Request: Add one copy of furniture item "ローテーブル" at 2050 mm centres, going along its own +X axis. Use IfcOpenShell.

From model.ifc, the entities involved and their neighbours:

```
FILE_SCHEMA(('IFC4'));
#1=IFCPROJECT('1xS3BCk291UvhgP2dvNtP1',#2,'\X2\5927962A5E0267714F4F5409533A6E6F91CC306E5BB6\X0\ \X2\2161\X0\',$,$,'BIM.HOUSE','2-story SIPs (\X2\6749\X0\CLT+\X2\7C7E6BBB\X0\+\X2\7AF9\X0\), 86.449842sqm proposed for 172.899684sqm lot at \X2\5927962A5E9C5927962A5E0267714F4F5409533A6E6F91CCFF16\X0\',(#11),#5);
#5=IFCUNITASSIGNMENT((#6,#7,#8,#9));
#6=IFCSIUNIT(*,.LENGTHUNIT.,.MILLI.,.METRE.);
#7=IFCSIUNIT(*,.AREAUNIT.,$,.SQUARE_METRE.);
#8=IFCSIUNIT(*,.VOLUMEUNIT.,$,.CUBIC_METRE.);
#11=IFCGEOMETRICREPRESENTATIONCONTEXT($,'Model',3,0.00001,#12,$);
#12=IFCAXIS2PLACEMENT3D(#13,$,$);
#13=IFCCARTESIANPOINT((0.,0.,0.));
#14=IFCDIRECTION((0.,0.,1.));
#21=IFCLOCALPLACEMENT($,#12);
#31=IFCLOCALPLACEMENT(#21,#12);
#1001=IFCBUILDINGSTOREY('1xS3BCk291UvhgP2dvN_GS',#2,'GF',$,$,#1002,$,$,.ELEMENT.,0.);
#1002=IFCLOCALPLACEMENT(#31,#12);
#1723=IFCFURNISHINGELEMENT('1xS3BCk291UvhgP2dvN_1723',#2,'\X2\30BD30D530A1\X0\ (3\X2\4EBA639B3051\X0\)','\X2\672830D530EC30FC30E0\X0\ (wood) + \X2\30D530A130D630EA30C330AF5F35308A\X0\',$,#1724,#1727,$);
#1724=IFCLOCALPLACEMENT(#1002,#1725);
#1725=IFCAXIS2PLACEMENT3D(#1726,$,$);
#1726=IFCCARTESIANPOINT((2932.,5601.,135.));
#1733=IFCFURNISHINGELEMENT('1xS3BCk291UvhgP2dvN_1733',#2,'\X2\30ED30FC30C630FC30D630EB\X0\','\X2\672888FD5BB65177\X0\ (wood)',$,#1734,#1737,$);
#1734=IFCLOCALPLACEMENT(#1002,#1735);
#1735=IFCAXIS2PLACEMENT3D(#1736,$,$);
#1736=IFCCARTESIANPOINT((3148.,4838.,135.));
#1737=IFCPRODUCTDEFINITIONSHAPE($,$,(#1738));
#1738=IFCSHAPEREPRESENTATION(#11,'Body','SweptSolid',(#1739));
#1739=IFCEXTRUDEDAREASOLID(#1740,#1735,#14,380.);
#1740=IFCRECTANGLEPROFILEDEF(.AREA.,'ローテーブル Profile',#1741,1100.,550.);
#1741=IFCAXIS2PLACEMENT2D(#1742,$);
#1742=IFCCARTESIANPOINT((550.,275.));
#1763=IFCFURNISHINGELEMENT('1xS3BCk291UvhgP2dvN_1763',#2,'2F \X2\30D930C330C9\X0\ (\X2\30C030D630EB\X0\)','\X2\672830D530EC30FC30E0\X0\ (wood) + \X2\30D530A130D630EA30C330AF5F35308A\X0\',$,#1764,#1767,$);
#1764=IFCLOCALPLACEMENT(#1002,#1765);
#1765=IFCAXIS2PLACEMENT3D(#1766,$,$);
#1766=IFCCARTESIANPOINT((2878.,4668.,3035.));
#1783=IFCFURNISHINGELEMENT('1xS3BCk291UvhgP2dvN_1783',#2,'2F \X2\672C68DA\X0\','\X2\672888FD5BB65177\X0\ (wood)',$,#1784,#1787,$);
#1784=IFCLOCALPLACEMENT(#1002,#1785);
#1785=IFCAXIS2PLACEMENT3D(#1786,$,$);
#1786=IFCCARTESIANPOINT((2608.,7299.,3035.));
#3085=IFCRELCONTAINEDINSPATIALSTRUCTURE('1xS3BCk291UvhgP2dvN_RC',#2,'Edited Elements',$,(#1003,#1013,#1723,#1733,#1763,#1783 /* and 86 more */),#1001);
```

```python
import ifcopenshell
import ifcopenshell.api.geometry
import ifcopenshell.api.root
import ifcopenshell.util.element
import ifcopenshell.util.placement

model = ifcopenshell.open("model.ifc")


def reuse_history(source, copy):
    """copy_class also copies each property set's owner history, people and application; keep the originals."""
    for rel in copy.IsDefinedBy:
        if rel.is_a("IfcRelDefinesByProperties") and (history := rel.RelatingPropertyDefinition.OwnerHistory):
            rel.RelatingPropertyDefinition.OwnerHistory = source.OwnerHistory
            ifcopenshell.util.element.remove_deep2(model, history)


source = model.by_id(1733)
base = ifcopenshell.util.placement.get_local_placement(source.ObjectPlacement)
step = base[:3, 0] * 2050.0

for i in range(1, 2):
    copy = ifcopenshell.api.root.copy_class(model, product=source)
    copy.Representation = ifcopenshell.util.element.copy_deep(
        model, source.Representation, exclude=["IfcGeometricRepresentationContext", "IfcRepresentationMap"]
    )
    reuse_history(source, copy)
    matrix = base.copy()
    matrix[:3, 3] += i * step
    print("added at", matrix[:3, 3].round(3) + 0.0)
    ifcopenshell.api.geometry.edit_object_placement(model, product=copy, matrix=matrix, is_si=False)

model.write("model_rev.ifc")
```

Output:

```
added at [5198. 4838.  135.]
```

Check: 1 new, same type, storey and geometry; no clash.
